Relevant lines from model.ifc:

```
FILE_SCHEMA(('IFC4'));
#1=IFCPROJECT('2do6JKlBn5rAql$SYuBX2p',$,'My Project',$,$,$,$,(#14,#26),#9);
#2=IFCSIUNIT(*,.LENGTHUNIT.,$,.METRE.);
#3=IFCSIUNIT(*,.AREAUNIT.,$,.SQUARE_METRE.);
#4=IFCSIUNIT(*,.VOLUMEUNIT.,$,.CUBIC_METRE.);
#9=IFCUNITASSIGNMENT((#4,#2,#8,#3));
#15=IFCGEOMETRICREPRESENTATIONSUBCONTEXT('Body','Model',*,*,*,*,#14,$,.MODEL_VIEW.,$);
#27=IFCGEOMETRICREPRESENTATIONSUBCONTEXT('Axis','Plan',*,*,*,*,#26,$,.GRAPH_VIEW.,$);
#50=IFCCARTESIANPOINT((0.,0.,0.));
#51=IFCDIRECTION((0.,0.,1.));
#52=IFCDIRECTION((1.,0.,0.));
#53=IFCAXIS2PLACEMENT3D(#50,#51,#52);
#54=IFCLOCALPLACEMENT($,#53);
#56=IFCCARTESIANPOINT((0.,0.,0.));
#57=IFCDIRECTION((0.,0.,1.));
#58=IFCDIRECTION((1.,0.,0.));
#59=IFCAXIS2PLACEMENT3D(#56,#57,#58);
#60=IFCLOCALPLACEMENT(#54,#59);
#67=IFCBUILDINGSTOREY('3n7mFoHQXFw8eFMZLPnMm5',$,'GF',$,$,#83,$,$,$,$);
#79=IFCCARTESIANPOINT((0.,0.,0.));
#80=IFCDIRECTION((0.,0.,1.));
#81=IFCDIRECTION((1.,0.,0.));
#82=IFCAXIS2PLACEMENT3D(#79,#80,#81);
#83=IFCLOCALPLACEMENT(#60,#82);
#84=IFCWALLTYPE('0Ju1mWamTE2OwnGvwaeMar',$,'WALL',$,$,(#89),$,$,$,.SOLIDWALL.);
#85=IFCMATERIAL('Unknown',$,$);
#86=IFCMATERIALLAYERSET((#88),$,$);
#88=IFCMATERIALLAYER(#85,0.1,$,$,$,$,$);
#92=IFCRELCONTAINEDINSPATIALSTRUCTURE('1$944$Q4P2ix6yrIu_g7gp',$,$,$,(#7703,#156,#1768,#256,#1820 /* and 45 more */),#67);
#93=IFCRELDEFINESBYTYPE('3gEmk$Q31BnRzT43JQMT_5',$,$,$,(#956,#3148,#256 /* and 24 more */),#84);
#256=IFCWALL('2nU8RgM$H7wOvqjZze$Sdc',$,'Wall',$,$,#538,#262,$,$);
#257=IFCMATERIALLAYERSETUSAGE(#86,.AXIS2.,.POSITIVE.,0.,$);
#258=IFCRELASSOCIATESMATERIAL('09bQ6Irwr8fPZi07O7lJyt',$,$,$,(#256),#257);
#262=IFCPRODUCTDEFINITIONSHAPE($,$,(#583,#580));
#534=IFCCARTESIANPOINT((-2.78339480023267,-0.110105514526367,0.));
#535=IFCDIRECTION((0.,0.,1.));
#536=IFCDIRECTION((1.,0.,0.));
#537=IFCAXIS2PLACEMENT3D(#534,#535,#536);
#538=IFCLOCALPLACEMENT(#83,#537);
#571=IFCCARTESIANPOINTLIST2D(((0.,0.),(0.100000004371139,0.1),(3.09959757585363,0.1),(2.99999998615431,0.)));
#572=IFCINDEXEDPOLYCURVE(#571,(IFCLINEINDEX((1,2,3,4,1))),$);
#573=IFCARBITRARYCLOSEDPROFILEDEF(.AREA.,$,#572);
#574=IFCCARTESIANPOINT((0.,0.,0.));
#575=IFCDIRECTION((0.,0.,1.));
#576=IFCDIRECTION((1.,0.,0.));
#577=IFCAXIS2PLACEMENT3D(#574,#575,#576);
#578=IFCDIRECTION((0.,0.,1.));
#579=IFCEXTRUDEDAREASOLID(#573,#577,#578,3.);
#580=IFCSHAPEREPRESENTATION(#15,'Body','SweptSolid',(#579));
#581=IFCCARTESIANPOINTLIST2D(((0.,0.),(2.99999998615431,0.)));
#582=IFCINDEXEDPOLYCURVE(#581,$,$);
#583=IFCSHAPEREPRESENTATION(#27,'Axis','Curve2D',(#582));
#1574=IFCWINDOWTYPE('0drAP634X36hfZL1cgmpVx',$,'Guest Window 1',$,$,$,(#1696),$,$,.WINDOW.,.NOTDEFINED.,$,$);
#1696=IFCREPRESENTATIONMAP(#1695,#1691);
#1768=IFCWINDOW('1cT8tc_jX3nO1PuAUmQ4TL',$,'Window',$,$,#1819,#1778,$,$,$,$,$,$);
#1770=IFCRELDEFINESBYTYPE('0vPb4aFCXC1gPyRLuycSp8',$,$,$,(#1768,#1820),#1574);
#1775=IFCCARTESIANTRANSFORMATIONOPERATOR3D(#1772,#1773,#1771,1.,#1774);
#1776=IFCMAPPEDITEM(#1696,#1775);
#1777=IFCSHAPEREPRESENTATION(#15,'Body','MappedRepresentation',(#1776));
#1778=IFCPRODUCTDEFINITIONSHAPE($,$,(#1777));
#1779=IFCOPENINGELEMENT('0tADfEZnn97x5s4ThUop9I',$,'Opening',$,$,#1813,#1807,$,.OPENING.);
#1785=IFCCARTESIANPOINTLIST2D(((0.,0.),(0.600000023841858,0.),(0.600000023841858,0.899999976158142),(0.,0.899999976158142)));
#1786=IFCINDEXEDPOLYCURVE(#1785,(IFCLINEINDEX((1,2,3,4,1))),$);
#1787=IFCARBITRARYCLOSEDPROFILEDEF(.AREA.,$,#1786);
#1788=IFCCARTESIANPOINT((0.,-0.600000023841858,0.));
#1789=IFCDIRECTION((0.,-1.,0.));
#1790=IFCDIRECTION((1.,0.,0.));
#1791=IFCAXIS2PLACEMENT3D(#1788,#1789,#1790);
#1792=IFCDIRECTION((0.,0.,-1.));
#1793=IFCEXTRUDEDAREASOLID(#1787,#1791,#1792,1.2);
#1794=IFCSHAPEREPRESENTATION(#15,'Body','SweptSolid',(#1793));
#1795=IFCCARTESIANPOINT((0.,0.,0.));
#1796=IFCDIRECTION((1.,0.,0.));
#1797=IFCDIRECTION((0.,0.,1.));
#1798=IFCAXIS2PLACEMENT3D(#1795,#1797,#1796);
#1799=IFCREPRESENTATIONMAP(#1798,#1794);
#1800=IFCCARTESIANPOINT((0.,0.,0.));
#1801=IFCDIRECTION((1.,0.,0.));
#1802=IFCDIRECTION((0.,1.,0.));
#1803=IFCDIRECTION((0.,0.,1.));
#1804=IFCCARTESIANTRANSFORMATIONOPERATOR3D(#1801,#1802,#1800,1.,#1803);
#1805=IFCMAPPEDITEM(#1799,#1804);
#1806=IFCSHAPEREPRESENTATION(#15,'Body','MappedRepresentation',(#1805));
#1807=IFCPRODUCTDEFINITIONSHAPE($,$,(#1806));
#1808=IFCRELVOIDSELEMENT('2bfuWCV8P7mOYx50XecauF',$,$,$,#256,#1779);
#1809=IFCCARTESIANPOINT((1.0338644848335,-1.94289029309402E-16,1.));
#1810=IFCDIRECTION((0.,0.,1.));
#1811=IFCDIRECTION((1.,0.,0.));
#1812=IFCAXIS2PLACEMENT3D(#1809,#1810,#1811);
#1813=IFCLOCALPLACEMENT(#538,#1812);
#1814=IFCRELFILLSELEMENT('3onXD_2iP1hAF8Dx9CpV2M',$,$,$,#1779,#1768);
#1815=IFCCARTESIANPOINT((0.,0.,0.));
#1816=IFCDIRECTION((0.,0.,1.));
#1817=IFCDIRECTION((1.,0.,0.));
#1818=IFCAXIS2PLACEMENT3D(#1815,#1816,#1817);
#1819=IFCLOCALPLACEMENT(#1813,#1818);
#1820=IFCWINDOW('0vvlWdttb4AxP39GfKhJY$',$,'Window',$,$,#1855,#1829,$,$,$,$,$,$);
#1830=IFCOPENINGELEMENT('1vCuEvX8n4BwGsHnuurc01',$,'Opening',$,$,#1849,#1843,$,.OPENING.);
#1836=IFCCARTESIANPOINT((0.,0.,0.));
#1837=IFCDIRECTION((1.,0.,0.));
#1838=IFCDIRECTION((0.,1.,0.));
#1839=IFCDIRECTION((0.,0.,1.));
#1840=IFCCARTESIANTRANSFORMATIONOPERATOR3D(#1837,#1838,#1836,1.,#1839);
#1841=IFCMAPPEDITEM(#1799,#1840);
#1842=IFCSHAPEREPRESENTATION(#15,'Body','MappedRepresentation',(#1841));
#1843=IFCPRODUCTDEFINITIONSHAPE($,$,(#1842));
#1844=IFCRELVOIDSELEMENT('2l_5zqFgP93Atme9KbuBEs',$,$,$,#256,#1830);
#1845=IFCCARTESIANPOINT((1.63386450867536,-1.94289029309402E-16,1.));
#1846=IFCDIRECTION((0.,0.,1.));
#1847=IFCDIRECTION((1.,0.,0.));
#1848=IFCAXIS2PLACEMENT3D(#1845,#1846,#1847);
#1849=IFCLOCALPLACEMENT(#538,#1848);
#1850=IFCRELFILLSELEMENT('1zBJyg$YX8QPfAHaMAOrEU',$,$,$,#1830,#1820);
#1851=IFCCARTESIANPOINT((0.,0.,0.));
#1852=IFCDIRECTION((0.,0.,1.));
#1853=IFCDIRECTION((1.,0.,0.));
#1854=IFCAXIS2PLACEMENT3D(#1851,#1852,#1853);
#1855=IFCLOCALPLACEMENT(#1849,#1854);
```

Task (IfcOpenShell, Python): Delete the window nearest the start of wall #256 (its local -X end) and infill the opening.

```python
import ifcopenshell
import ifcopenshell.api.feature
import ifcopenshell.api.root
import ifcopenshell.geom
import ifcopenshell.util.shape

model = ifcopenshell.open("model.ifc")
settings = ifcopenshell.geom.settings()


def volume(element):
    """Net volume in cubic metres, openings subtracted."""
    shape = ifcopenshell.geom.create_shape(settings, element)
    return ifcopenshell.util.shape.get_volume(shape.geometry)


window = model.by_guid("1cT8tc_jX3nO1PuAUmQ4TL")
opening = window.FillsVoids[0].RelatingOpeningElement
wall = opening.VoidsElements[0].RelatingBuildingElement
before = volume(wall)

ifcopenshell.api.root.remove_product(model, product=window)
ifcopenshell.api.feature.remove_feature(model, feature=opening)

after = volume(wall)

print(f"wall volume {before:.3f} -> {after:.3f} m3")

model.write("model_updated.ifc")
```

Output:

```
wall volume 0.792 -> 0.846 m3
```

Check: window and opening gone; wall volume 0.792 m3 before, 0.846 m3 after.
